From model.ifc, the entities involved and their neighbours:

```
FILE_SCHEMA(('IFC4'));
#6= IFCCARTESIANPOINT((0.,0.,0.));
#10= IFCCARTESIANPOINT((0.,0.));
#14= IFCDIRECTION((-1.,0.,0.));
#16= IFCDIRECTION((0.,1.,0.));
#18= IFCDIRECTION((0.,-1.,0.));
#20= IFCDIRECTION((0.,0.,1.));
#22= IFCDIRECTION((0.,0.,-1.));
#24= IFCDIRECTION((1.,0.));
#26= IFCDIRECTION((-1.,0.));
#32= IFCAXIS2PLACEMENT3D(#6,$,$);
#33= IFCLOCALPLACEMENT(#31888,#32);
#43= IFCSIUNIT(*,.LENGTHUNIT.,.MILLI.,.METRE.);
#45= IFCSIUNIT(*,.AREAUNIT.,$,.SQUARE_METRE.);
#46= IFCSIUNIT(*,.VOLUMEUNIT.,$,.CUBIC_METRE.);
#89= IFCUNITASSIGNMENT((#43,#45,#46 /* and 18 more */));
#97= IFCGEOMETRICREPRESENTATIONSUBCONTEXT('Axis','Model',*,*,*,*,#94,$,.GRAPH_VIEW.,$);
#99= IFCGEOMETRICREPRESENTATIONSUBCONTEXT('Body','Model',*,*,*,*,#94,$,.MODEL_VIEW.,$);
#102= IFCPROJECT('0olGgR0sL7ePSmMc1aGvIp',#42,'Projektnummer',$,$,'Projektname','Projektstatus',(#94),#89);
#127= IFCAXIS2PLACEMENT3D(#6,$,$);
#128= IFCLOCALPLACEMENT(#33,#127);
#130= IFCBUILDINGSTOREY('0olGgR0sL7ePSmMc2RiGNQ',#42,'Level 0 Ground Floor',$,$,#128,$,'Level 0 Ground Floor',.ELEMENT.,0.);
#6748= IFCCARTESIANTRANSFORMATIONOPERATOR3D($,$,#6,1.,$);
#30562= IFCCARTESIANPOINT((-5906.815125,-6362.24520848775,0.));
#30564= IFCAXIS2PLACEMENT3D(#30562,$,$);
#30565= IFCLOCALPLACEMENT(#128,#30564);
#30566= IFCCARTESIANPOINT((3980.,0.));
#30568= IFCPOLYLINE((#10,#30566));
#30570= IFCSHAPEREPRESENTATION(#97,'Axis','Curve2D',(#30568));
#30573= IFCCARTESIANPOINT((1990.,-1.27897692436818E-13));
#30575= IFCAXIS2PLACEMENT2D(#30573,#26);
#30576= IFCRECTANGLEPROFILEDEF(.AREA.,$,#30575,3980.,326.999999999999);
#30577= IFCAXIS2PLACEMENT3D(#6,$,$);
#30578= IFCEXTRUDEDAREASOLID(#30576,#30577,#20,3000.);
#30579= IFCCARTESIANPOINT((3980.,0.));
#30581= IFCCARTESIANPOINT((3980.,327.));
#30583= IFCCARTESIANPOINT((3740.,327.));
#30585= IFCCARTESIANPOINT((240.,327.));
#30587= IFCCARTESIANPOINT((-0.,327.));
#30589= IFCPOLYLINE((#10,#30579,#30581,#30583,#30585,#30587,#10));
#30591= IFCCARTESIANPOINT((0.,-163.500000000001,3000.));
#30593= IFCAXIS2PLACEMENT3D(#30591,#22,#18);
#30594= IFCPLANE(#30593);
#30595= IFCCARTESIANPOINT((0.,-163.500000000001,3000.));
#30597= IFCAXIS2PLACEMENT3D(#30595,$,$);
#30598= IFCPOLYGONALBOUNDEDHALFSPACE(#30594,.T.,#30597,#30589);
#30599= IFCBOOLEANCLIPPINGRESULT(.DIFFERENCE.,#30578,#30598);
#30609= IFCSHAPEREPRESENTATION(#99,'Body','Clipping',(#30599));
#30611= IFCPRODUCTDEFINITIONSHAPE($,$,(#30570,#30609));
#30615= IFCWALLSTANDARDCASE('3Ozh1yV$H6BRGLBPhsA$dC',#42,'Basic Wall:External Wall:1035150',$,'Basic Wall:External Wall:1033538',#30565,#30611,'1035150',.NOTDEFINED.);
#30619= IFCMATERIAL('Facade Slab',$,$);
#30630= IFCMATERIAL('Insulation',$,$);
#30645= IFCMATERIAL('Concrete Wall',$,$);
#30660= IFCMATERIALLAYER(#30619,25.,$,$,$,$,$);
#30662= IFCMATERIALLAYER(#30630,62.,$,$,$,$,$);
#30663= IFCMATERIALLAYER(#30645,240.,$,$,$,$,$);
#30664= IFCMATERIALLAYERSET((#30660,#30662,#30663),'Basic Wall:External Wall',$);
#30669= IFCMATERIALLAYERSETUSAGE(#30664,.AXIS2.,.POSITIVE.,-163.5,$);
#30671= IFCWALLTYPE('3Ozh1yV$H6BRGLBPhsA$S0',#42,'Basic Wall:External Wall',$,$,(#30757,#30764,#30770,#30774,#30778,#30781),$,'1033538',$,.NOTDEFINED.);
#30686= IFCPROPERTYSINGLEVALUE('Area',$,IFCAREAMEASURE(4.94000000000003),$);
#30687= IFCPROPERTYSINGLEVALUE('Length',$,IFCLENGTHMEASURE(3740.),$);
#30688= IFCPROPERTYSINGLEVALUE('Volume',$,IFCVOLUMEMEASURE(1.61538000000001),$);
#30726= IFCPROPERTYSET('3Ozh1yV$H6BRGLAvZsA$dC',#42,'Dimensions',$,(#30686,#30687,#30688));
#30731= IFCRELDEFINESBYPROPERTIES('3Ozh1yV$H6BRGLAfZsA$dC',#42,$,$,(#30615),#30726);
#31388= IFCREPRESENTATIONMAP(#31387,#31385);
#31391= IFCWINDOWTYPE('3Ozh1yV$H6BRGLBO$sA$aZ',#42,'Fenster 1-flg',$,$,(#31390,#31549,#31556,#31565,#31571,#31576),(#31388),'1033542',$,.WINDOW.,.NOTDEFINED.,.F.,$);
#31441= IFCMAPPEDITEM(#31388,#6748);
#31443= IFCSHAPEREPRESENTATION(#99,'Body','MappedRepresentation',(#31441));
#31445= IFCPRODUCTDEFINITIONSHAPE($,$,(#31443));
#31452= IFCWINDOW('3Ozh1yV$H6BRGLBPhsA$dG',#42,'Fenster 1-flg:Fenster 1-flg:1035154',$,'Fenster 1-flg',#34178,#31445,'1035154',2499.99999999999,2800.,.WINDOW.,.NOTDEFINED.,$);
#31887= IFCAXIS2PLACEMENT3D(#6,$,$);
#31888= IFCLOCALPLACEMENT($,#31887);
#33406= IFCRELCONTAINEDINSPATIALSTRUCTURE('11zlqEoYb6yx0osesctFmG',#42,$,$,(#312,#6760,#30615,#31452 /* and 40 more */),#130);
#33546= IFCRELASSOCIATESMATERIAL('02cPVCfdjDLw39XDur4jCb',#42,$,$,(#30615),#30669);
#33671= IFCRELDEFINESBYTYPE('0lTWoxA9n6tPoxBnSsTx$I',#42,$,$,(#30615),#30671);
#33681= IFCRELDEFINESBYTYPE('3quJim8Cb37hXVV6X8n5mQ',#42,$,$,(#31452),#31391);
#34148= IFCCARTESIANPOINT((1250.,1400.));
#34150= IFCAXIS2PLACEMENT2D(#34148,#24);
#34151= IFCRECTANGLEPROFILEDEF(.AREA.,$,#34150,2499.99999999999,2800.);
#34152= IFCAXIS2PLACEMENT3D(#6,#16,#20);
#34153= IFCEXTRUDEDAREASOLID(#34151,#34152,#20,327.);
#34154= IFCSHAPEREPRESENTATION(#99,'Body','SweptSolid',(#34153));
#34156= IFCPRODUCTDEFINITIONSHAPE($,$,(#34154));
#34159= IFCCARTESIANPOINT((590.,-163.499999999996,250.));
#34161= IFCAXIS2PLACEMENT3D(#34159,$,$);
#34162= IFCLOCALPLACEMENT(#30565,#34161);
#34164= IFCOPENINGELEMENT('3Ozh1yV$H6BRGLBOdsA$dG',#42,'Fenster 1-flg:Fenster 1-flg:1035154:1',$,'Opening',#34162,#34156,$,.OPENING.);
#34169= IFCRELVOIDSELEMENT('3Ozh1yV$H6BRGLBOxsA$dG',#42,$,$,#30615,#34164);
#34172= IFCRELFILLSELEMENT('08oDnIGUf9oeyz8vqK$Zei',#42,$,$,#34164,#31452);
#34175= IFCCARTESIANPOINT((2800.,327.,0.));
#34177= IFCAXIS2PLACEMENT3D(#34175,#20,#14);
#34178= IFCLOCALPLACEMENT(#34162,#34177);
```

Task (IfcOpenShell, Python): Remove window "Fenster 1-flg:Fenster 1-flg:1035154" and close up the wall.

```python
import ifcopenshell
import ifcopenshell.api.feature
import ifcopenshell.api.pset
import ifcopenshell.api.root
import ifcopenshell.geom
import ifcopenshell.util.element
import ifcopenshell.util.shape
import ifcopenshell.util.unit

model = ifcopenshell.open("model.ifc")
area_scale = ifcopenshell.util.unit.calculate_unit_scale(model, "AREAUNIT")
volume_scale = ifcopenshell.util.unit.calculate_unit_scale(model, "VOLUMEUNIT")
settings = ifcopenshell.geom.settings()


def volume(element):
    """Net volume in cubic metres, openings subtracted."""
    shape = ifcopenshell.geom.create_shape(settings, element)
    return ifcopenshell.util.shape.get_volume(shape.geometry)


window = model.by_guid("3Ozh1yV$H6BRGLBPhsA$dG")
opening = window.FillsVoids[0].RelatingOpeningElement
wall = opening.VoidsElements[0].RelatingBuildingElement
before = volume(wall)

ifcopenshell.api.root.remove_product(model, product=window)
ifcopenshell.api.feature.remove_feature(model, feature=opening)

after = volume(wall)
thickness = 0.327  # wall thickness in metres

# Update the wall's stored quantities.
pset = model.by_id(ifcopenshell.util.element.get_pset(wall, "Dimensions", should_inherit=False)["id"])
ifcopenshell.api.pset.edit_pset(model, pset=pset, properties={
    "Area": model.create_entity("IfcAreaMeasure", after / thickness / area_scale),
    "Volume": model.create_entity("IfcVolumeMeasure", after / volume_scale),
})

print(f"wall volume {before:.3f} -> {after:.3f} m3")

model.write("model_rev.ifc")
```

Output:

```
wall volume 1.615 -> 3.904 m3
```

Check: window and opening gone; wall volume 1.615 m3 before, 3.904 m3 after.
